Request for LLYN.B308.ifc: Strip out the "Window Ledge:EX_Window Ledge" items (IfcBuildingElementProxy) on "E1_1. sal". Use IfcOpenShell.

First a look at what the model holds.

```python
import ifcopenshell
import ifcopenshell.util.element

model = ifcopenshell.open("LLYN.B308.ifc")
print(model.schema)
storey = next(s for s in model.by_type("IfcBuildingStorey") if s.Name == "E1_1. sal")
proxies = [e for e in ifcopenshell.util.element.get_decomposition(storey) if e.is_a("IfcBuildingElementProxy")]
seen = {}
for e in proxies:
    element_type = ifcopenshell.util.element.get_type(e)
    name = element_type.Name if element_type not in (None, e) else None
    seen[name] = seen.get(name, 0) + 1
for name, count in sorted(seen.items(), key=str):
    print(count, "x", name)
```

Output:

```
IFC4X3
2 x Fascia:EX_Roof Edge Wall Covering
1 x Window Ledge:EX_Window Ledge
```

```python
import ifcopenshell
import ifcopenshell.api.root
import ifcopenshell.util.element

model = ifcopenshell.open("LLYN.B308.ifc")

storey = next(s for s in model.by_type("IfcBuildingStorey") if s.Name == "E1_1. sal")
proxies = [e for e in ifcopenshell.util.element.get_decomposition(storey) if e.is_a("IfcBuildingElementProxy")]
targets = [e for e in proxies if (t := ifcopenshell.util.element.get_type(e)) not in (None, e) and t.Name == "Window Ledge:EX_Window Ledge"]

for e in targets:
    ifcopenshell.api.root.remove_product(model, product=e)
print(len(targets), "removed")

model.write("LLYN.B308_edited.ifc")
```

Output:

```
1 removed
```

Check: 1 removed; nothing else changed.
